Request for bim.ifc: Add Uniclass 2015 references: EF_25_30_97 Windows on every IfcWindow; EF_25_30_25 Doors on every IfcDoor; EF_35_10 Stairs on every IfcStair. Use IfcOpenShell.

First a look at what the model holds.

```python
import ifcopenshell

model = ifcopenshell.open("bim.ifc")
print(model.schema)
print("classifications:", [c.Name for c in model.by_type("IfcClassification")])
for ifc_class in ("IfcDoor", "IfcRoof", "IfcStair", "IfcWall", "IfcWindow"):
    print(ifc_class, len(model.by_type(ifc_class)))
```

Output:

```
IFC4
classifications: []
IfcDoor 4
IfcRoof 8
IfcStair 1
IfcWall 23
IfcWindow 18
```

```python
import ifcopenshell
import ifcopenshell.api.classification

model = ifcopenshell.open("bim.ifc")

system = ifcopenshell.api.classification.add_classification(model, classification="Uniclass 2015")

codes = {
    "IfcWindow": ("EF_25_30_97", "Windows"),
    "IfcDoor": ("EF_25_30_25", "Doors"),
    "IfcStair": ("EF_35_10", "Stairs"),
}
for ifc_class, (code, name) in codes.items():
    products = model.by_type(ifc_class)
    ifcopenshell.api.classification.add_reference(
        model, products=products, classification=system, identification=code, name=name
    )
    print(code, len(products))

model.write("bim_rev.ifc")
```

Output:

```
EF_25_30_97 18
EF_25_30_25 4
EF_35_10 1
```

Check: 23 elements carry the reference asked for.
